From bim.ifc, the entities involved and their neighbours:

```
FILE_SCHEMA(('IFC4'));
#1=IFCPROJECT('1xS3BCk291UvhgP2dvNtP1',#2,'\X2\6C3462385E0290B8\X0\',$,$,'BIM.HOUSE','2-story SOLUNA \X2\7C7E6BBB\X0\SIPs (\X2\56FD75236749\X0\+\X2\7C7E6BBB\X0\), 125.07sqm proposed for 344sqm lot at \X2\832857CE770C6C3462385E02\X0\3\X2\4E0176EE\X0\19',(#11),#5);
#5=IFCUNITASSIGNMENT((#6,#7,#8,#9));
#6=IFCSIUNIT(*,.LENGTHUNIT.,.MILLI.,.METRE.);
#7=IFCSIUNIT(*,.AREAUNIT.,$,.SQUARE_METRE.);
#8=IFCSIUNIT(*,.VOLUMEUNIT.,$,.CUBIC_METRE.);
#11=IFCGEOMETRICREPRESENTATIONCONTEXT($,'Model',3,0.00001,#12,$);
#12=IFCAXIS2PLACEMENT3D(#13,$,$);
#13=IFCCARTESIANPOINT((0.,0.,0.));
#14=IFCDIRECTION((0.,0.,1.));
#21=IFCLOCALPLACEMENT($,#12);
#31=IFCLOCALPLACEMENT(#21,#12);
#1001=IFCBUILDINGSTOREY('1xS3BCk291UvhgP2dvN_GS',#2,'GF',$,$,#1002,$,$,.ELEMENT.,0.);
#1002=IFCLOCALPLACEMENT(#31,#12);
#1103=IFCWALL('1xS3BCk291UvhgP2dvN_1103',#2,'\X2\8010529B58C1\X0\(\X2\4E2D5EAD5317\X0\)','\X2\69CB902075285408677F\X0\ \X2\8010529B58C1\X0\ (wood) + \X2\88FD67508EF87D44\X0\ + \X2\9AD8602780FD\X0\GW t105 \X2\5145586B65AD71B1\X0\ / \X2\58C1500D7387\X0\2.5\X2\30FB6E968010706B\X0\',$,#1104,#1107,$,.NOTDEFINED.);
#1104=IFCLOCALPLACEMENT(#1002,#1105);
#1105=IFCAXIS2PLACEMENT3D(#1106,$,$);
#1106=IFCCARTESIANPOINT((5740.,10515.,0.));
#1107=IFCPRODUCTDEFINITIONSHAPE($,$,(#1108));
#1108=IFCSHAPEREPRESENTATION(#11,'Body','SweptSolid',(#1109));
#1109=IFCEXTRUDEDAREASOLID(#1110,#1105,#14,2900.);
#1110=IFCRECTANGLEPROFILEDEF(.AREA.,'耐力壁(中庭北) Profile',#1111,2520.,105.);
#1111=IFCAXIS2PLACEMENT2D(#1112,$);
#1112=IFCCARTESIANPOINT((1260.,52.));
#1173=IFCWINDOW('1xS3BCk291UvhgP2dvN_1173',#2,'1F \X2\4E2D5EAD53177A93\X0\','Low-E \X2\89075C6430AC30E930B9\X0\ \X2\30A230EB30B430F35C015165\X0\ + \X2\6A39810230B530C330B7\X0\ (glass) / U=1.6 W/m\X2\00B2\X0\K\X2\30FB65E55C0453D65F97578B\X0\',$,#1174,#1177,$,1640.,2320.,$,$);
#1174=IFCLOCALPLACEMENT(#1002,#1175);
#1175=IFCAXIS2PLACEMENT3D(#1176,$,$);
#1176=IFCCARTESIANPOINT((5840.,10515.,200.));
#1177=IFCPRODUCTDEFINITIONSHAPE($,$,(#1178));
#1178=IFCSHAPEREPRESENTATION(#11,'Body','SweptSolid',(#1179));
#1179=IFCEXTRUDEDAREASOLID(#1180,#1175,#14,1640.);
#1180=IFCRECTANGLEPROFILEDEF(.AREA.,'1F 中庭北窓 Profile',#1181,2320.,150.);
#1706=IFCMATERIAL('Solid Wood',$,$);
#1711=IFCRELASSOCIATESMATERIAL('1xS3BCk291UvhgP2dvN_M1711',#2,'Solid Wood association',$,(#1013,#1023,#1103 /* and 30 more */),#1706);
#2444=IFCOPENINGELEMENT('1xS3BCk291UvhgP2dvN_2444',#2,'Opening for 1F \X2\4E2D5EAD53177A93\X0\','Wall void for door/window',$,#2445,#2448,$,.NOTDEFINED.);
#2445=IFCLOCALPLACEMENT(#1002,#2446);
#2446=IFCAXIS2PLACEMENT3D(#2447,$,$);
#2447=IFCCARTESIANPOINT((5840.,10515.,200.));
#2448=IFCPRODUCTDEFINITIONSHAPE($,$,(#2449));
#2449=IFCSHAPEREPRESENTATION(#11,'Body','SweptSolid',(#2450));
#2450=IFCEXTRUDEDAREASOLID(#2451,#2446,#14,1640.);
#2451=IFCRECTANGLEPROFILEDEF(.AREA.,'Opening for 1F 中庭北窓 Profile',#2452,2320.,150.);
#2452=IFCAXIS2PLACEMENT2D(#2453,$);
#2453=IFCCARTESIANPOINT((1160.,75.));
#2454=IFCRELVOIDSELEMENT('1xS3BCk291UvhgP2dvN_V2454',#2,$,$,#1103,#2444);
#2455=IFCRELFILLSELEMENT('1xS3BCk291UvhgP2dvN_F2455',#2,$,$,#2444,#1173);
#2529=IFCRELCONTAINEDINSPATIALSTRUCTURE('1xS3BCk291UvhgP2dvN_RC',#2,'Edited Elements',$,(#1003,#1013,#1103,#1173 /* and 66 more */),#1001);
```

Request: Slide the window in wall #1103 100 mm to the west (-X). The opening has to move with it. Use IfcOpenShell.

```python
import ifcopenshell
import ifcopenshell.api.geometry
import ifcopenshell.util.placement

model = ifcopenshell.open("bim.ifc")

window = model.by_guid("1xS3BCk291UvhgP2dvN_1173")
opening = window.FillsVoids[0].RelatingOpeningElement
wall = opening.VoidsElements[0].RelatingBuildingElement

wall_matrix = ifcopenshell.util.placement.get_local_placement(wall.ObjectPlacement)
shift = wall_matrix[:3, 0] * -100.0
before = ifcopenshell.util.placement.get_local_placement(window.ObjectPlacement)[:3, 3].copy()

# The window is not placed relative to its opening, so move both.
for product in (opening, window):
    matrix = ifcopenshell.util.placement.get_local_placement(product.ObjectPlacement)
    matrix[:3, 3] += shift
    ifcopenshell.api.geometry.edit_object_placement(model, product=product, matrix=matrix, is_si=False)

after = ifcopenshell.util.placement.get_local_placement(window.ObjectPlacement)[:3, 3]
print("window moved by", (after - before).round(3) + 0.0)

model.write("bim_v2.ifc")
```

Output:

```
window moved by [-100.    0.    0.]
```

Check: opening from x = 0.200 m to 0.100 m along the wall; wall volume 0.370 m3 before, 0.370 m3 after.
